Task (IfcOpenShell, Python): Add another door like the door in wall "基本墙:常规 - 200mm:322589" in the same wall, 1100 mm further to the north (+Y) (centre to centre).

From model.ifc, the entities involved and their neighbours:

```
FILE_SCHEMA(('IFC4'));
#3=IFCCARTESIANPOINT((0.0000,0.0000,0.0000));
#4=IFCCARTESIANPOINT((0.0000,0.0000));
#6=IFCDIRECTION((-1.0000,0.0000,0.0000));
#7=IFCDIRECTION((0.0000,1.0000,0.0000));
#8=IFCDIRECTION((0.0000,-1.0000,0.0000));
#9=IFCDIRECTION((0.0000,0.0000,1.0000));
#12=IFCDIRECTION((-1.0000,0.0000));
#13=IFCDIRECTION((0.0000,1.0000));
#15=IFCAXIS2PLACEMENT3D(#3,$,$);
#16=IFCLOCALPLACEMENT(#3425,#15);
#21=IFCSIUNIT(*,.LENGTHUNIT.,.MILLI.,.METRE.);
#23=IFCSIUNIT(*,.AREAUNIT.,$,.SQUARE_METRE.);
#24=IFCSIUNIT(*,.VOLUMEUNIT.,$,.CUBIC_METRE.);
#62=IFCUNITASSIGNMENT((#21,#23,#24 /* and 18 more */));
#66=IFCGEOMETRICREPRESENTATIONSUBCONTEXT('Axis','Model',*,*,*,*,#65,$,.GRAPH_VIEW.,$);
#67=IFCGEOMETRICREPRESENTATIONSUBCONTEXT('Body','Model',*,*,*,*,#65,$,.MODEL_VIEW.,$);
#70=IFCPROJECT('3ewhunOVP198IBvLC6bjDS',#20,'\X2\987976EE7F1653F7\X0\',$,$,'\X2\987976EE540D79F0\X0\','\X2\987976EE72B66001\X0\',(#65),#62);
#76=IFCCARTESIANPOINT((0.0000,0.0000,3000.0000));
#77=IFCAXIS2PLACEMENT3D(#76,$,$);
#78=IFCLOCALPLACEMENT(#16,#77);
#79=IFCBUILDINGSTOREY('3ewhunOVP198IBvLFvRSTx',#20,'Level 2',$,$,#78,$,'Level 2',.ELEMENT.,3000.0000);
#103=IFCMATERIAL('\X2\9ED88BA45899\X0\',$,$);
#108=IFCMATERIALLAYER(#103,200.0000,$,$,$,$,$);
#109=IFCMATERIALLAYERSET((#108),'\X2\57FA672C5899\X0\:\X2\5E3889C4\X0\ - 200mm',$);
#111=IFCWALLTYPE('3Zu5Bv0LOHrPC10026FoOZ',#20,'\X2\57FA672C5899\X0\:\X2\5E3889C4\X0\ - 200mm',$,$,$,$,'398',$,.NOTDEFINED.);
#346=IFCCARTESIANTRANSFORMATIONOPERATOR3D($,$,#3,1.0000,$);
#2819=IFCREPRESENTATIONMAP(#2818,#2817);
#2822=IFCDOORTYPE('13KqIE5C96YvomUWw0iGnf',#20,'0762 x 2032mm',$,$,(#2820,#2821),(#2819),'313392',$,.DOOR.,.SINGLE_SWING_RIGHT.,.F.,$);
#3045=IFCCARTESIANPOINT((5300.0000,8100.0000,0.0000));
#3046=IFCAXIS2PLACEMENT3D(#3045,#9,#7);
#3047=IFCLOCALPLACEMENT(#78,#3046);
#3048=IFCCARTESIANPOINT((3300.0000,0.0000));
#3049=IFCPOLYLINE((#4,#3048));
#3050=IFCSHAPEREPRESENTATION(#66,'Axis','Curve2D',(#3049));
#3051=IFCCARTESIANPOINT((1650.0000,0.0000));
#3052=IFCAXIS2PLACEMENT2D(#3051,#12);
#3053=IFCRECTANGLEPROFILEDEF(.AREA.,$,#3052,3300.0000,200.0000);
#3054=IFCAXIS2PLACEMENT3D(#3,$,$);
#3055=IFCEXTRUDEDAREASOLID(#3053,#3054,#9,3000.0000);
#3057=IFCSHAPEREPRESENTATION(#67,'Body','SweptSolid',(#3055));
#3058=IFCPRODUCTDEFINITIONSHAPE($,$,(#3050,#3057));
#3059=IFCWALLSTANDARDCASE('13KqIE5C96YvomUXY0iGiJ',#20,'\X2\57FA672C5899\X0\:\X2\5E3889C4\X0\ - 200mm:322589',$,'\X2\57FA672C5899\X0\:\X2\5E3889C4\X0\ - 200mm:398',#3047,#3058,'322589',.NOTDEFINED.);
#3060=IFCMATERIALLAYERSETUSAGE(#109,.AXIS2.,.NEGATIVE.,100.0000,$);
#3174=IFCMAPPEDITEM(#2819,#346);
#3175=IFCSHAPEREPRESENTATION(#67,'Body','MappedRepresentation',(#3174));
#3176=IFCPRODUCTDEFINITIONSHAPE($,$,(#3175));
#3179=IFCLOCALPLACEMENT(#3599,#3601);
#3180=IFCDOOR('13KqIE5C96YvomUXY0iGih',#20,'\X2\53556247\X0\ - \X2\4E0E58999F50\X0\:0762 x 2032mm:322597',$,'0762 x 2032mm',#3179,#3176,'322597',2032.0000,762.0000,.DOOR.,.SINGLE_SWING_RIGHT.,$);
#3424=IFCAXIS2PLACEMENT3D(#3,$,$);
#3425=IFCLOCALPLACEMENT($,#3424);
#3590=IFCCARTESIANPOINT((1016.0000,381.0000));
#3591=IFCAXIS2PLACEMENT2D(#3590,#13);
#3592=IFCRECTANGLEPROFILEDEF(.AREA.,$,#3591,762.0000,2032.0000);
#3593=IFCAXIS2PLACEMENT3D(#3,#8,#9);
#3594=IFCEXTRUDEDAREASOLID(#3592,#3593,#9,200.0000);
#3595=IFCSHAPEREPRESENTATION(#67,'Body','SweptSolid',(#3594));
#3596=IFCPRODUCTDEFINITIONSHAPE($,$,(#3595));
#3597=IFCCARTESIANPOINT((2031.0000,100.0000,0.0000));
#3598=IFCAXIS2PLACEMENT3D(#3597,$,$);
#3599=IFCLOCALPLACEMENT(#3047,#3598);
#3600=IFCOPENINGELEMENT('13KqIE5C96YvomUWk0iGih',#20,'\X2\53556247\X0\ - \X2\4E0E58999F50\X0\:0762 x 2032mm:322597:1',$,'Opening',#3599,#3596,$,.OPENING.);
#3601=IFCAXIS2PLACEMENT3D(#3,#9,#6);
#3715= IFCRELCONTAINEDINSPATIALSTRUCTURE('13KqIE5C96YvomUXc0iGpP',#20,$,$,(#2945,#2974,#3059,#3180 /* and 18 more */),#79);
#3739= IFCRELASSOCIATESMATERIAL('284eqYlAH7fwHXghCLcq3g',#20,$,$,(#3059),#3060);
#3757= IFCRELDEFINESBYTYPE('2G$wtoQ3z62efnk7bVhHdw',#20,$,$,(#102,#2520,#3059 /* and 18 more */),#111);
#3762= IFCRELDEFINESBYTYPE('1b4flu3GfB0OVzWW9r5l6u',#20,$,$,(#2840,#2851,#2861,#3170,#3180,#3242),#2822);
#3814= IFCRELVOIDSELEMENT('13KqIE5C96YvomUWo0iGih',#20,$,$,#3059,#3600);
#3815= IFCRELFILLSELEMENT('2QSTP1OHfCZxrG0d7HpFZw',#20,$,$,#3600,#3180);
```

```python
import ifcopenshell
import ifcopenshell.api.feature
import ifcopenshell.api.geometry
import ifcopenshell.api.root
import ifcopenshell.geom
import ifcopenshell.util.element
import ifcopenshell.util.placement
import ifcopenshell.util.shape

model = ifcopenshell.open("model.ifc")
settings = ifcopenshell.geom.settings()


def volume(element):
    """Net volume in cubic metres, openings subtracted."""
    shape = ifcopenshell.geom.create_shape(settings, element)
    return ifcopenshell.util.shape.get_volume(shape.geometry)


def reuse_history(source, copy):
    """copy_class also copies each property set's owner history, people and application; keep the originals."""
    for rel in copy.IsDefinedBy:
        if rel.is_a("IfcRelDefinesByProperties") and (history := rel.RelatingPropertyDefinition.OwnerHistory):
            rel.RelatingPropertyDefinition.OwnerHistory = source.OwnerHistory
            ifcopenshell.util.element.remove_deep2(model, history)


door = model.by_guid("13KqIE5C96YvomUXY0iGih")
opening = door.FillsVoids[0].RelatingOpeningElement
wall = opening.VoidsElements[0].RelatingBuildingElement
before = volume(wall)
shift = ifcopenshell.util.placement.get_local_placement(wall.ObjectPlacement)[:3, 0] * 1100.0

# copy_class copies the void relationship, type, container and properties, but no geometry.
new_opening = ifcopenshell.api.root.copy_class(model, product=opening)
new_opening.Representation = ifcopenshell.util.element.copy_deep(
    model, opening.Representation, exclude=["IfcGeometricRepresentationContext", "IfcRepresentationMap"]
)
new_opening.Name = "单扇 - 与墙齐:0762 x 2032mm"
new_door = ifcopenshell.api.root.copy_class(model, product=door)
new_door.Representation = ifcopenshell.util.element.copy_deep(
    model, door.Representation, exclude=["IfcGeometricRepresentationContext", "IfcRepresentationMap"]
)
new_door.Name = "单扇 - 与墙齐:0762 x 2032mm"
new_door.Tag = None
reuse_history(door, new_door)
ifcopenshell.api.feature.add_filling(model, opening=new_opening, element=new_door)

for old, new in ((opening, new_opening), (door, new_door)):
    matrix = ifcopenshell.util.placement.get_local_placement(old.ObjectPlacement)
    matrix[:3, 3] += shift
    ifcopenshell.api.geometry.edit_object_placement(model, product=new, matrix=matrix, is_si=False)

after = volume(wall)

print(f"wall volume {before:.3f} -> {after:.3f} m3")

model.write("model_edited.ifc")
```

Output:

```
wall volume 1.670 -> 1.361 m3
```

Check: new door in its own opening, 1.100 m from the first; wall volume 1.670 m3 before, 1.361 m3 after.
